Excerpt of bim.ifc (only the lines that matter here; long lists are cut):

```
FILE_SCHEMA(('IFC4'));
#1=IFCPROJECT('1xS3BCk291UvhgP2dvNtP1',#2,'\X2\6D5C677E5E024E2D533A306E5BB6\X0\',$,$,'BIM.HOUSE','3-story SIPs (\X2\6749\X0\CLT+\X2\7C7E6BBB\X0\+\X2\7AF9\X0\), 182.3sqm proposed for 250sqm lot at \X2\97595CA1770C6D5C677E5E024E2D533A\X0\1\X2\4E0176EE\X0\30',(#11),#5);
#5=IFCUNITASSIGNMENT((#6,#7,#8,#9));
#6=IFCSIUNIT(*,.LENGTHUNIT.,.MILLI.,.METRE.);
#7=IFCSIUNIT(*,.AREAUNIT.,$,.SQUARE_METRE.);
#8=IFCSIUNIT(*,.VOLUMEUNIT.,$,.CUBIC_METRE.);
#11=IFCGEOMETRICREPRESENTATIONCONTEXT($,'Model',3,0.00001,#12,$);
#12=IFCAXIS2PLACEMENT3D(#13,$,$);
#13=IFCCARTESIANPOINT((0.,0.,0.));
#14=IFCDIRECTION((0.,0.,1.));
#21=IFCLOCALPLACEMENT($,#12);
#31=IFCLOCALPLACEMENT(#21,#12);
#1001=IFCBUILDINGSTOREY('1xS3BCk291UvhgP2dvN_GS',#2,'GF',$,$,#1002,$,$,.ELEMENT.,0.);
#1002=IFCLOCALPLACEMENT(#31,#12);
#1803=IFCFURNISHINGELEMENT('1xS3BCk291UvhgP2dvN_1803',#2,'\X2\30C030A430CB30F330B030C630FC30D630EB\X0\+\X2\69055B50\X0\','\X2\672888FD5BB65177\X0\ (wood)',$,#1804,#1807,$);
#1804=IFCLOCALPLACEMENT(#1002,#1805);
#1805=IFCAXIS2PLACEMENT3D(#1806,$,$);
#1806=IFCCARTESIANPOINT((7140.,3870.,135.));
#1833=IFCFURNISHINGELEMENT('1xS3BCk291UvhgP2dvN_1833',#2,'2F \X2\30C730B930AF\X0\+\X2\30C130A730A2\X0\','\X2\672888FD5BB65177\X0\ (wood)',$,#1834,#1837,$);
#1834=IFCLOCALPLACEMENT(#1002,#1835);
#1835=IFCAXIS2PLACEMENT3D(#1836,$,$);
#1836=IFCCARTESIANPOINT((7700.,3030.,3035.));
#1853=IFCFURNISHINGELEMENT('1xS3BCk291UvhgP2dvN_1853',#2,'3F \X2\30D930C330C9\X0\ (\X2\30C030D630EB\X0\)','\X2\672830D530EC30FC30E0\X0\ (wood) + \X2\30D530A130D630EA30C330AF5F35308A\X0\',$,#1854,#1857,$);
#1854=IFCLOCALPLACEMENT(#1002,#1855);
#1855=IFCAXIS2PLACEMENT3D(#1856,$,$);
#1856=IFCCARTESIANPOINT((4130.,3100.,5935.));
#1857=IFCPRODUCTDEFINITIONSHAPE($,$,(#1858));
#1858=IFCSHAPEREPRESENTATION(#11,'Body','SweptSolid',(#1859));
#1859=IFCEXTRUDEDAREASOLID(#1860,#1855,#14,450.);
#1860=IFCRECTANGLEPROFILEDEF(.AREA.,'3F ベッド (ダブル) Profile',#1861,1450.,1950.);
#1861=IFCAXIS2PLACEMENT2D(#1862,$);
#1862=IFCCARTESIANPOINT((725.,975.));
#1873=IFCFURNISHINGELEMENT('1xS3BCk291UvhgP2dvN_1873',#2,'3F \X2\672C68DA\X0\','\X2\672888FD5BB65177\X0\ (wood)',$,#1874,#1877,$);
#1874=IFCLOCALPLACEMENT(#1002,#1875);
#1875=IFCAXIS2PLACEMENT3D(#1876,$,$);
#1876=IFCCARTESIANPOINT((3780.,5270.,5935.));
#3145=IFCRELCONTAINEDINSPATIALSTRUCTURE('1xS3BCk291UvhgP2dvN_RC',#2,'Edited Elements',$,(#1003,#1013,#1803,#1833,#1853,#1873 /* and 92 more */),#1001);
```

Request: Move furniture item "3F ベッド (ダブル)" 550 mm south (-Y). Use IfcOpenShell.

```python
import ifcopenshell
import ifcopenshell.api.geometry
import ifcopenshell.util.placement
import ifcopenshell.util.unit

model = ifcopenshell.open("bim.ifc")
unit_scale = ifcopenshell.util.unit.calculate_unit_scale(model)

item = model.by_id(1853)
matrix = ifcopenshell.util.placement.get_local_placement(item.ObjectPlacement)
matrix[1, 3] -= 0.55 / unit_scale
ifcopenshell.api.geometry.edit_object_placement(model, product=item, matrix=matrix, is_si=False)

print(ifcopenshell.util.placement.get_local_placement(item.ObjectPlacement).round(3) + 0.0)

model.write("bim_edited.ifc")
```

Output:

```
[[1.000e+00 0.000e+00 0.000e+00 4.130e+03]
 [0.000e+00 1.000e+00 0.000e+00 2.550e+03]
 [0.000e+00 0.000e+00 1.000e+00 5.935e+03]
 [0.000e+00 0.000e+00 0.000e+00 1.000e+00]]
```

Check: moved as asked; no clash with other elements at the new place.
